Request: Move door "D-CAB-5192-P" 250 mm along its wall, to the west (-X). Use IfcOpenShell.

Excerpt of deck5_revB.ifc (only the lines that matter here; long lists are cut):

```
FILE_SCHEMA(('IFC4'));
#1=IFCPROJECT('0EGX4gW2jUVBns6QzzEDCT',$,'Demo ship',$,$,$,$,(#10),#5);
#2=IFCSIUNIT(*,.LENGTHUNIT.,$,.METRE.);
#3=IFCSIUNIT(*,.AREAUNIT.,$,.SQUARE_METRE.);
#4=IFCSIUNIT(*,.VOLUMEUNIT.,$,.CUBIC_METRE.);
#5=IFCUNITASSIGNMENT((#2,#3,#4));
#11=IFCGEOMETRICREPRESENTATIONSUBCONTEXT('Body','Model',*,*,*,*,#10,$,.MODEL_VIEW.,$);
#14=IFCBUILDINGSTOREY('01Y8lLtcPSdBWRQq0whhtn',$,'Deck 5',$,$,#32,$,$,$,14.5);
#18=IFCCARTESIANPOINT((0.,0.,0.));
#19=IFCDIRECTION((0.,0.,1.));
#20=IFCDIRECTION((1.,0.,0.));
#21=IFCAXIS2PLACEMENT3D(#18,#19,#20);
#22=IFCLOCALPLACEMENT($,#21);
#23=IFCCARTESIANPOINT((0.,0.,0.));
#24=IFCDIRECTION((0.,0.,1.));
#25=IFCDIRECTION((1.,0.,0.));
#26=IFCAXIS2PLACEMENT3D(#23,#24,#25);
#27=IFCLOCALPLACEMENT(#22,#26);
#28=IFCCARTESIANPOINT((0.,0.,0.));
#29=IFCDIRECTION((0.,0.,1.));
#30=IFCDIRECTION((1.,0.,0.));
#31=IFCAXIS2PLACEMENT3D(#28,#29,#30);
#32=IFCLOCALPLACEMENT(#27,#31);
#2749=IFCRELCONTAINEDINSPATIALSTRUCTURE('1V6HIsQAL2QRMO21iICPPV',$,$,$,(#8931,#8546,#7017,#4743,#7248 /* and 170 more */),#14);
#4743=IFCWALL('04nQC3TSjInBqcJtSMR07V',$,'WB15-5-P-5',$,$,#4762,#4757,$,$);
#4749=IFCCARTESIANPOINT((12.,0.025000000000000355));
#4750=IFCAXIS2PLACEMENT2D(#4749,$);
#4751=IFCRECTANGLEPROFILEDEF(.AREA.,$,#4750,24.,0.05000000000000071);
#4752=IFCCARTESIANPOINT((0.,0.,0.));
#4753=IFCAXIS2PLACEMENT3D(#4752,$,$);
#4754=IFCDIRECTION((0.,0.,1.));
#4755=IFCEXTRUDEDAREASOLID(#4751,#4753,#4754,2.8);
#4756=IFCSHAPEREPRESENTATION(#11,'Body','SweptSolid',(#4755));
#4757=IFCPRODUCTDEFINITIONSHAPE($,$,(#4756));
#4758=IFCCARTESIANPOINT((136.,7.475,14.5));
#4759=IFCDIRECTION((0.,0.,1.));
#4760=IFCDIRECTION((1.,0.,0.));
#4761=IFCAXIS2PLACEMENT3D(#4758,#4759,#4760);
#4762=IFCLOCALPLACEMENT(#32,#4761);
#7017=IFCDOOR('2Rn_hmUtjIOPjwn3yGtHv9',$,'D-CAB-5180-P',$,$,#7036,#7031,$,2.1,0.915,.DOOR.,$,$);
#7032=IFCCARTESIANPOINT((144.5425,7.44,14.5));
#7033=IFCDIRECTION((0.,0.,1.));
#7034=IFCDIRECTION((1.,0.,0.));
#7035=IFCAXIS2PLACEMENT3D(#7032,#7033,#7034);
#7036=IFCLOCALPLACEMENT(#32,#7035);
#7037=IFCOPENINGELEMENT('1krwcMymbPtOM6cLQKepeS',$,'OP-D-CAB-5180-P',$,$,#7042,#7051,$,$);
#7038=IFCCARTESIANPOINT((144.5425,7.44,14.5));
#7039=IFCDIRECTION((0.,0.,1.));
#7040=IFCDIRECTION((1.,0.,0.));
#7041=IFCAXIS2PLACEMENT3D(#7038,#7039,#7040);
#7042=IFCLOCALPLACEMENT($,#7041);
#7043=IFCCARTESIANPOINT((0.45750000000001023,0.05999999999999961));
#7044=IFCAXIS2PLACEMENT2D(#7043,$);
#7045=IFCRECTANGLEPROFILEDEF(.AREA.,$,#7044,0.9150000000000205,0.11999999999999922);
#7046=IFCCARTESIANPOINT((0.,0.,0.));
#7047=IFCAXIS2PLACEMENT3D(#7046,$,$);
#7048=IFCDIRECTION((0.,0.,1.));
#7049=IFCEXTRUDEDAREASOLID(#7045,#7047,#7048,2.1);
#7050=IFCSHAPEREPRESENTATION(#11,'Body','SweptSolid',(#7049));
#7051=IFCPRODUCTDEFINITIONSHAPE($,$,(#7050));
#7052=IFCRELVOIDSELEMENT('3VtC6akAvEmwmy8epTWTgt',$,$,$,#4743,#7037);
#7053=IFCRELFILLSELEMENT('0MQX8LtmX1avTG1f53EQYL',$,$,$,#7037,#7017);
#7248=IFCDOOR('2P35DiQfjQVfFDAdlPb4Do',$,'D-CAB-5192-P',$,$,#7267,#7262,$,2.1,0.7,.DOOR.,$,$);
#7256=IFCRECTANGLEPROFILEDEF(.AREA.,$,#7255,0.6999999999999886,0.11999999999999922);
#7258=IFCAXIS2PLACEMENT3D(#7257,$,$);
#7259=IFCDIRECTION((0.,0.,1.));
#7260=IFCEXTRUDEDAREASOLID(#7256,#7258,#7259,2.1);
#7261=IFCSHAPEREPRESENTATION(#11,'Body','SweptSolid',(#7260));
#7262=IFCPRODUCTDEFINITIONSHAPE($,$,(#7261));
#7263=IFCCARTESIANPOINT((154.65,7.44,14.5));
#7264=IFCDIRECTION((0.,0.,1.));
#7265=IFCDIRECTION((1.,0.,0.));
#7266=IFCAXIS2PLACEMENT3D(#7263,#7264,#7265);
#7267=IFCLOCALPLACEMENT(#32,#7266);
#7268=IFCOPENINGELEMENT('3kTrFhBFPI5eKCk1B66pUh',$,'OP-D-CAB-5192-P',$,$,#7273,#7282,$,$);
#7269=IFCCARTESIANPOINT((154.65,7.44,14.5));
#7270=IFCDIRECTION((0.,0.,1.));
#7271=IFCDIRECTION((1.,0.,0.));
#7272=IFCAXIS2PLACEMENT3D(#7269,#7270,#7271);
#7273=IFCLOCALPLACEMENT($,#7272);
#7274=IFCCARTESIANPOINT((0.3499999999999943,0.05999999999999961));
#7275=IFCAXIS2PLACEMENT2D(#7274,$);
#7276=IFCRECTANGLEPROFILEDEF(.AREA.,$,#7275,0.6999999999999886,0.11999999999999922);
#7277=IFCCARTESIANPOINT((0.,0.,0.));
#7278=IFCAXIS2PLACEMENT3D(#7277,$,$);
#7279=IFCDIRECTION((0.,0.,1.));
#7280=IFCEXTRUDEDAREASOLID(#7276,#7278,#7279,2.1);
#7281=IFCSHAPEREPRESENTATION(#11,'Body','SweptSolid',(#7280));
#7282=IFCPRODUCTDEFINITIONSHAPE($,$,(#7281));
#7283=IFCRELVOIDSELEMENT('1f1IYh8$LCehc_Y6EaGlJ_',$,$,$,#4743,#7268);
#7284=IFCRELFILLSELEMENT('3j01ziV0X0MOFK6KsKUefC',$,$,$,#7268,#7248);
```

```python
import ifcopenshell
import ifcopenshell.api.geometry
import ifcopenshell.util.placement

model = ifcopenshell.open("deck5_revB.ifc")

door = model.by_guid("2P35DiQfjQVfFDAdlPb4Do")
opening = door.FillsVoids[0].RelatingOpeningElement
wall = opening.VoidsElements[0].RelatingBuildingElement

wall_matrix = ifcopenshell.util.placement.get_local_placement(wall.ObjectPlacement)
shift = wall_matrix[:3, 0] * -0.25
before = ifcopenshell.util.placement.get_local_placement(door.ObjectPlacement)[:3, 3].copy()

# The door is not placed relative to its opening, so move both.
for product in (opening, door):
    matrix = ifcopenshell.util.placement.get_local_placement(product.ObjectPlacement)
    matrix[:3, 3] += shift
    ifcopenshell.api.geometry.edit_object_placement(model, product=product, matrix=matrix, is_si=False)

after = ifcopenshell.util.placement.get_local_placement(door.ObjectPlacement)[:3, 3]
print("door moved by", (after - before).round(3) + 0.0)

model.write("deck5_revB_v2.ifc")
```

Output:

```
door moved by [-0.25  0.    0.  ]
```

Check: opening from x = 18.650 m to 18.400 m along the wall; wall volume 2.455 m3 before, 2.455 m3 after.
